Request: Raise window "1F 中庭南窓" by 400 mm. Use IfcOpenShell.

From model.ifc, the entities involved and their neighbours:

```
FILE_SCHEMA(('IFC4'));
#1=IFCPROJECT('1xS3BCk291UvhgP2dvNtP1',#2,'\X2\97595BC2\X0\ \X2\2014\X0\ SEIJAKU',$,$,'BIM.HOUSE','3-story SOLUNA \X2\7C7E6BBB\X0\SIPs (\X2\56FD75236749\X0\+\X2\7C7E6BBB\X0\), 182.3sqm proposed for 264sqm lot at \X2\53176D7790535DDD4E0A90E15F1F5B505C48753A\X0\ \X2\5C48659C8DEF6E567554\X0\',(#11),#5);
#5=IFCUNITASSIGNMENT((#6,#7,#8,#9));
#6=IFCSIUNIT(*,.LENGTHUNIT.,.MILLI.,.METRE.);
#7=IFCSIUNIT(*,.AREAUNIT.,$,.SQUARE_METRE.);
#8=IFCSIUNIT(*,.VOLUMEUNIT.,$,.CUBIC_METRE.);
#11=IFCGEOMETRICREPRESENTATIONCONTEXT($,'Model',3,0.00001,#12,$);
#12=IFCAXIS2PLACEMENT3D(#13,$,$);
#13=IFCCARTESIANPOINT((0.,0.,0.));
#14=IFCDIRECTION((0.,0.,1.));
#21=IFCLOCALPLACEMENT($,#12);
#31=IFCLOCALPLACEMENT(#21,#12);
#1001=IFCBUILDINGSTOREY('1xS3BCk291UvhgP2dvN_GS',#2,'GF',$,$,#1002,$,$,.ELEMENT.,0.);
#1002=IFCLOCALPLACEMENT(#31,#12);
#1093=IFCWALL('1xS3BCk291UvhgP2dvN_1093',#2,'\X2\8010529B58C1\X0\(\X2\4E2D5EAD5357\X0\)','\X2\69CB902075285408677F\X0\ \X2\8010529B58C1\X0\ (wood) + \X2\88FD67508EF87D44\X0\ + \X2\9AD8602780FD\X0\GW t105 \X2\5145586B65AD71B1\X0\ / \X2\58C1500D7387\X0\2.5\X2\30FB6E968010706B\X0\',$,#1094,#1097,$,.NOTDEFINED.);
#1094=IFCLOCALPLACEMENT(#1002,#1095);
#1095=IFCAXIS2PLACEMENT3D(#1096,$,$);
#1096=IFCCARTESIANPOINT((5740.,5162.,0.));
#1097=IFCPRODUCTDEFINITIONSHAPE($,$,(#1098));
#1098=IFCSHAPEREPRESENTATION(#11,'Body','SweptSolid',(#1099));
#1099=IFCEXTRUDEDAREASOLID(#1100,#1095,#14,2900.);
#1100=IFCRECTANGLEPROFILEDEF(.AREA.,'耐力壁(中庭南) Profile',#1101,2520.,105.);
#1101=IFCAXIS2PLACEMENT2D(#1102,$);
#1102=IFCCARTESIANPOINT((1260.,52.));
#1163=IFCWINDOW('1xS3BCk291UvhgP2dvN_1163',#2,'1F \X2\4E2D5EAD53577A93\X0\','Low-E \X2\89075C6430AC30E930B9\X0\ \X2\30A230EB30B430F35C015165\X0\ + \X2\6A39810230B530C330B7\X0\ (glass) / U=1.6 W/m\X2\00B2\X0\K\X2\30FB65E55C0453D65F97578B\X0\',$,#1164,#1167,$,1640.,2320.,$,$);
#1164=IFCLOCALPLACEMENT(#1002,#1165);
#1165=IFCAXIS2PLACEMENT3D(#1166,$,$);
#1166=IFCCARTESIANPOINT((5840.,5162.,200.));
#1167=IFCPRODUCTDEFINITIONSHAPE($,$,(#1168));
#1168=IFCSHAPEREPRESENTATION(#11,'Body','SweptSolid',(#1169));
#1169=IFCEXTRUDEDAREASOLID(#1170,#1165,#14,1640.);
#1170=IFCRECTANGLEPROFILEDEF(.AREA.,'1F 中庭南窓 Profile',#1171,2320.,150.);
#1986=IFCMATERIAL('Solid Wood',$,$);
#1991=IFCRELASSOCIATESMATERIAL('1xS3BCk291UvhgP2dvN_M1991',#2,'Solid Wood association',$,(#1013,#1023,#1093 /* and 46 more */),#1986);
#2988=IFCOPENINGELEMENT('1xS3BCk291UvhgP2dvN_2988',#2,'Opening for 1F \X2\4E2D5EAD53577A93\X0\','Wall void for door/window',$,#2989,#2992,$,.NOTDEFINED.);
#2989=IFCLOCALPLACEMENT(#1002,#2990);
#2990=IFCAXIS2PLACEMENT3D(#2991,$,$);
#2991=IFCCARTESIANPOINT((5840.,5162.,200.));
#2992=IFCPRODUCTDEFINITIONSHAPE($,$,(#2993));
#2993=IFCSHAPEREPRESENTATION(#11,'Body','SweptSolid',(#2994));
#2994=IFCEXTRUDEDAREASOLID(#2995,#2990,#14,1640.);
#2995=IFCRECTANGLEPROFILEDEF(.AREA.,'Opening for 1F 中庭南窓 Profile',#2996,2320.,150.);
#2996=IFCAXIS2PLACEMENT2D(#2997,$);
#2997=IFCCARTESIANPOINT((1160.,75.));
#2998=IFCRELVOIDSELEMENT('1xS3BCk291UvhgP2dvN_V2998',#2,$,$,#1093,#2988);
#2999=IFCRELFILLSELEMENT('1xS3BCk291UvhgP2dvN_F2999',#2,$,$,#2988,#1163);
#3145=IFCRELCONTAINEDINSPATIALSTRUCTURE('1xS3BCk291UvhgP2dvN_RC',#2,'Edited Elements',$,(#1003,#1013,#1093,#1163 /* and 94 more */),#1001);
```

```python
import numpy as np
import ifcopenshell
import ifcopenshell.api.geometry
import ifcopenshell.util.placement
import ifcopenshell.util.unit

model = ifcopenshell.open("model.ifc")
unit_scale = ifcopenshell.util.unit.calculate_unit_scale(model)

window = model.by_guid("1xS3BCk291UvhgP2dvN_1163")
opening = window.FillsVoids[0].RelatingOpeningElement
dz = 400.0

shift = np.array([0.0, 0.0, dz])
# The window is not placed relative to its opening, so move both.
for product in (opening, window):
    matrix = ifcopenshell.util.placement.get_local_placement(product.ObjectPlacement)
    matrix[:3, 3] += shift
    ifcopenshell.api.geometry.edit_object_placement(model, product=product, matrix=matrix, is_si=False)

print(f"moved by {dz * unit_scale:+.3f} m")

model.write("model_edited.ifc")
```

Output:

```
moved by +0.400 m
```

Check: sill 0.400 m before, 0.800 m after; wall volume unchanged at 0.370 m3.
